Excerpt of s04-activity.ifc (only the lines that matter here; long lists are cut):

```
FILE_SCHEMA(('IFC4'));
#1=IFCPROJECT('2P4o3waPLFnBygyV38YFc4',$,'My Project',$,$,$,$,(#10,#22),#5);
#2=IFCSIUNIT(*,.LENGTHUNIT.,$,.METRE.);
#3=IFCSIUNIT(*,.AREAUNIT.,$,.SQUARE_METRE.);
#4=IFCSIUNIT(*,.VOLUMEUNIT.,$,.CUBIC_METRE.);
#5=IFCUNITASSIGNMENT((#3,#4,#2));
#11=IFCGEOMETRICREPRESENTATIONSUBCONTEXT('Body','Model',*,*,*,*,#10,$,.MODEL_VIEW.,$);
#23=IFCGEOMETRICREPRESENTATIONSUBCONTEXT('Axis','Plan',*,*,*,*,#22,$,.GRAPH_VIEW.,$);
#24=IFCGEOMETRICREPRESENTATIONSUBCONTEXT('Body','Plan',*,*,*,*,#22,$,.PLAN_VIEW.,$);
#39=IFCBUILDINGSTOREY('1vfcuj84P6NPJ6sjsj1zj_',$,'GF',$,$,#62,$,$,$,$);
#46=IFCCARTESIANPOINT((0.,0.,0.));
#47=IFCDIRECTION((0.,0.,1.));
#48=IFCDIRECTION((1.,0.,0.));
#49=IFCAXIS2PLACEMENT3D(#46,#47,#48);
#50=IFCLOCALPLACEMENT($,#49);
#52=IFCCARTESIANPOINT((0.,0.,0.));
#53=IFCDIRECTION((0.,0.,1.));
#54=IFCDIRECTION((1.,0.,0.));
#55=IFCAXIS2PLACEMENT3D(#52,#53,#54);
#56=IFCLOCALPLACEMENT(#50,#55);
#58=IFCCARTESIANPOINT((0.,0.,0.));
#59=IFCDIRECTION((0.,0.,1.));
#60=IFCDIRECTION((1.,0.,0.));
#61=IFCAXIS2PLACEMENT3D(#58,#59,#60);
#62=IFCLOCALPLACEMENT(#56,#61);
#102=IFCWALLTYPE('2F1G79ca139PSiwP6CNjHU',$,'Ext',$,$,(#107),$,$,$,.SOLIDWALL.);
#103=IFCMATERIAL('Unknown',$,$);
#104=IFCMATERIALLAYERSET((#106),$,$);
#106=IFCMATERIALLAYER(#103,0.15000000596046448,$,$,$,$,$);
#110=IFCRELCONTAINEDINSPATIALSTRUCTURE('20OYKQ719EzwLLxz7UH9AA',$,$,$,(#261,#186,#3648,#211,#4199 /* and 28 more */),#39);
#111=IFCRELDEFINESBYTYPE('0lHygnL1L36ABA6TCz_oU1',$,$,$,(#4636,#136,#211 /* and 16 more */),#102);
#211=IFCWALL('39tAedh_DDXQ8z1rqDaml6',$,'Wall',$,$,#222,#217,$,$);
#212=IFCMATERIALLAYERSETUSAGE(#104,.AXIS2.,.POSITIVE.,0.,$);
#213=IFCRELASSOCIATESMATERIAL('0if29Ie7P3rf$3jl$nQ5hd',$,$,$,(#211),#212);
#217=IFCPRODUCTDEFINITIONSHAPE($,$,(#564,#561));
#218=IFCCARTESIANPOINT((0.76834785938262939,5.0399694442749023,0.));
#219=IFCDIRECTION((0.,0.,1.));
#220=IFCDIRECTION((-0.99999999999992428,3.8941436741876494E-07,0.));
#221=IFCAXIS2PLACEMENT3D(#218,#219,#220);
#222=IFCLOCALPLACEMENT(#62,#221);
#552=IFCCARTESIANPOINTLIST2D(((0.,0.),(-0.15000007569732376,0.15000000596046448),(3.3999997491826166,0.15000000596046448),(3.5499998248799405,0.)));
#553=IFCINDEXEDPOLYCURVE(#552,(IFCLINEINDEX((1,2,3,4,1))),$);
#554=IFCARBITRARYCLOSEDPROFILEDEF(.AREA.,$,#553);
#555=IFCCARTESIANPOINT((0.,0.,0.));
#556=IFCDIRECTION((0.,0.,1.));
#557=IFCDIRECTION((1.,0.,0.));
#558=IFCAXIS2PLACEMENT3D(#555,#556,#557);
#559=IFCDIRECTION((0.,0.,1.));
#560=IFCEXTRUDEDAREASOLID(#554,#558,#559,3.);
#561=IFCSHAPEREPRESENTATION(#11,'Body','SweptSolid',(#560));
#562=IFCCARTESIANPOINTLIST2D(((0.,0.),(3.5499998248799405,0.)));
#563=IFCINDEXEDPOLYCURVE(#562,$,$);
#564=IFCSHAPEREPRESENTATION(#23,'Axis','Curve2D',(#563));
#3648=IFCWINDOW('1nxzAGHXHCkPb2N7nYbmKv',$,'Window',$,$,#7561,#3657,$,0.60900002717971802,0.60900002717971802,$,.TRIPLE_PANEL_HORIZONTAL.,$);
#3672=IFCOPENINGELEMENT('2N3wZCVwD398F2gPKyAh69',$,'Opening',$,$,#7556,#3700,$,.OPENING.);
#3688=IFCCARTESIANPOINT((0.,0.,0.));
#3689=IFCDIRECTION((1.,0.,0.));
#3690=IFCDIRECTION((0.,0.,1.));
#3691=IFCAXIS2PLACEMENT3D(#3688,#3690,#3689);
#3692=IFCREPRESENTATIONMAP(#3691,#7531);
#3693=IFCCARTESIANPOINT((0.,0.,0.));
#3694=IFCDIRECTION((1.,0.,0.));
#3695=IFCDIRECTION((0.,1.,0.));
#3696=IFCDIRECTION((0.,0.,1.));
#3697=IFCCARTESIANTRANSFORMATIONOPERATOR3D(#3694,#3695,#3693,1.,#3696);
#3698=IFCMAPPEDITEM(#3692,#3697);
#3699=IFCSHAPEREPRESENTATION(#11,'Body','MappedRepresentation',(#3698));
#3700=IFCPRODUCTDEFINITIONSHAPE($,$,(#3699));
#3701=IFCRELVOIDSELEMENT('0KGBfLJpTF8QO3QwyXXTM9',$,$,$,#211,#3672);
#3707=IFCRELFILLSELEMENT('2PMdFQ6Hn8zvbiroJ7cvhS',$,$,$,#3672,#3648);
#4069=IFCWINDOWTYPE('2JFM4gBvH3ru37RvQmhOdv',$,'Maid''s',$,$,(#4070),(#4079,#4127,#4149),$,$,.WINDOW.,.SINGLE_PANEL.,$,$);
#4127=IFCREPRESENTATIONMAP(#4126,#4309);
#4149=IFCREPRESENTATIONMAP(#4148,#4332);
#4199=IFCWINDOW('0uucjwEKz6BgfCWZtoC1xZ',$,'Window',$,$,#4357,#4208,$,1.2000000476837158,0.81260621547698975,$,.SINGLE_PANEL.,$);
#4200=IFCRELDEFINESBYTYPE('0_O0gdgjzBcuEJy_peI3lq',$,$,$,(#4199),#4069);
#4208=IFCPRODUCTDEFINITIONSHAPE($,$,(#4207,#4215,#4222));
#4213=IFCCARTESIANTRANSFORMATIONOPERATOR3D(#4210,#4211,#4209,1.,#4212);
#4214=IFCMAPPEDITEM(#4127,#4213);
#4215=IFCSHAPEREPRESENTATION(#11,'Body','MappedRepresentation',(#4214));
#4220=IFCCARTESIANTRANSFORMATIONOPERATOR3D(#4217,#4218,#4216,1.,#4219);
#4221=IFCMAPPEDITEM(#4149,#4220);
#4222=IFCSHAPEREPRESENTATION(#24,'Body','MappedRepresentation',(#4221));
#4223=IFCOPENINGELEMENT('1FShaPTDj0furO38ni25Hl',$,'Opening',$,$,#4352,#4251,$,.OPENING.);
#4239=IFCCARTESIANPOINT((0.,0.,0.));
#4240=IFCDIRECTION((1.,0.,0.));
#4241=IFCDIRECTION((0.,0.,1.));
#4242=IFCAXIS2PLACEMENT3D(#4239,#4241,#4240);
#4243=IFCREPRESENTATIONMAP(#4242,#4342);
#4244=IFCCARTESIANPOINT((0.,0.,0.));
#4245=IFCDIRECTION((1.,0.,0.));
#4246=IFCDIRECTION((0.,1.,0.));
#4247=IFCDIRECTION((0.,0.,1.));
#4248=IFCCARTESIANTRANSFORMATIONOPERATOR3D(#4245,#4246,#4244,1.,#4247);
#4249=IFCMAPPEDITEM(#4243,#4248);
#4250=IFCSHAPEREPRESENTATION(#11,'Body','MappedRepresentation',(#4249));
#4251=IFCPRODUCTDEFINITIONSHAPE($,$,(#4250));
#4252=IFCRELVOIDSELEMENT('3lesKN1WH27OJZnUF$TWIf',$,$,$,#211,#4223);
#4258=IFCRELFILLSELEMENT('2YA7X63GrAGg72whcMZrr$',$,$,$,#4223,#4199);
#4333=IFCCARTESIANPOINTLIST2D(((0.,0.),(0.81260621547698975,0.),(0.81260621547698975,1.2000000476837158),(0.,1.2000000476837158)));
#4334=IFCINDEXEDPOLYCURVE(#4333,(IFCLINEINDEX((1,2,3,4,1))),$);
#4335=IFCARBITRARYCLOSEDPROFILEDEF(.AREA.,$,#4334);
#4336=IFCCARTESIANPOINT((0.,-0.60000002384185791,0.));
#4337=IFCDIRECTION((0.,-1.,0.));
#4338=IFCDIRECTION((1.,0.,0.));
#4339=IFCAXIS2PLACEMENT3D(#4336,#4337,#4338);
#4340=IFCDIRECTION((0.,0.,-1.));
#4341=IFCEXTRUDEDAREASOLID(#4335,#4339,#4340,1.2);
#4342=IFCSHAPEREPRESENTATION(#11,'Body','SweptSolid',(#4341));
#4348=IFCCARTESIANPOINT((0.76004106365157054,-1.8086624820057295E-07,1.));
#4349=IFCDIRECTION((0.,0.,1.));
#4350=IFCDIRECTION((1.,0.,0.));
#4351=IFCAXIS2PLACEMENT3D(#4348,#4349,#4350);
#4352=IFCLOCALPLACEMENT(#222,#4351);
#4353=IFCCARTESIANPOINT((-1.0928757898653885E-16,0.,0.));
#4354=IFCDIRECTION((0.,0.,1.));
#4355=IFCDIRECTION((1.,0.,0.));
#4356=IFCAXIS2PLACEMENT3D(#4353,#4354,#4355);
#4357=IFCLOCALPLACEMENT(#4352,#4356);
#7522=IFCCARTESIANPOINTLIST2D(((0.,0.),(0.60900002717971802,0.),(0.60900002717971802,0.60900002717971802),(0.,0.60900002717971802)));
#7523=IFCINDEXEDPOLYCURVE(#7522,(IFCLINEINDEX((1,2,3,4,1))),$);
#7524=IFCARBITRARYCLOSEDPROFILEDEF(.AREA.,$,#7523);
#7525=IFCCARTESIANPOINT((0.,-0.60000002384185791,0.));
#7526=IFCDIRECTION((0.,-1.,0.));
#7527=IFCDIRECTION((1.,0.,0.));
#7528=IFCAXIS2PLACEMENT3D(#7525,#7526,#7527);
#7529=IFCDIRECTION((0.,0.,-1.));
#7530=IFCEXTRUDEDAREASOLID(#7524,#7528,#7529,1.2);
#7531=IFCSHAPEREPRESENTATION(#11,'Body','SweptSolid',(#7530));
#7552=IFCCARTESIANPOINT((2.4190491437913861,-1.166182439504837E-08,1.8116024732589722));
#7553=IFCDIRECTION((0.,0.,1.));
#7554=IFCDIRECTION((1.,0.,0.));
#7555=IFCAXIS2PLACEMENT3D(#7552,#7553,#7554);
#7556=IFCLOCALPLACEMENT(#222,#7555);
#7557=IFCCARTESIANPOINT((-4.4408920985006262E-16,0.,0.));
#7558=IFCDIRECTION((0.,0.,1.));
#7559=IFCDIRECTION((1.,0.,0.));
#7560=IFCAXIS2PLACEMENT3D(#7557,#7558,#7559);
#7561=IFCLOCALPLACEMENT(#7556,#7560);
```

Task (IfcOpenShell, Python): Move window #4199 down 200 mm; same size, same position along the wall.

```python
import numpy as np
import ifcopenshell
import ifcopenshell.api.geometry
import ifcopenshell.util.placement
import ifcopenshell.util.unit

model = ifcopenshell.open("s04-activity.ifc")
unit_scale = ifcopenshell.util.unit.calculate_unit_scale(model)

window = model.by_id(4199)
opening = window.FillsVoids[0].RelatingOpeningElement
dz = -0.2 / unit_scale

shift = np.array([0.0, 0.0, dz])
# The window is placed relative to its opening, so it follows when the opening moves.
matrix = ifcopenshell.util.placement.get_local_placement(opening.ObjectPlacement)
matrix[:3, 3] += shift
ifcopenshell.api.geometry.edit_object_placement(
    model, product=opening, matrix=matrix, is_si=False, should_transform_children=True
)

print(f"moved by {dz * unit_scale:+.3f} m")

model.write("s04-activity-out.ifc")
```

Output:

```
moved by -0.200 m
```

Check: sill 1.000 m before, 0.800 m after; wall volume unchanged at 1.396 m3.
